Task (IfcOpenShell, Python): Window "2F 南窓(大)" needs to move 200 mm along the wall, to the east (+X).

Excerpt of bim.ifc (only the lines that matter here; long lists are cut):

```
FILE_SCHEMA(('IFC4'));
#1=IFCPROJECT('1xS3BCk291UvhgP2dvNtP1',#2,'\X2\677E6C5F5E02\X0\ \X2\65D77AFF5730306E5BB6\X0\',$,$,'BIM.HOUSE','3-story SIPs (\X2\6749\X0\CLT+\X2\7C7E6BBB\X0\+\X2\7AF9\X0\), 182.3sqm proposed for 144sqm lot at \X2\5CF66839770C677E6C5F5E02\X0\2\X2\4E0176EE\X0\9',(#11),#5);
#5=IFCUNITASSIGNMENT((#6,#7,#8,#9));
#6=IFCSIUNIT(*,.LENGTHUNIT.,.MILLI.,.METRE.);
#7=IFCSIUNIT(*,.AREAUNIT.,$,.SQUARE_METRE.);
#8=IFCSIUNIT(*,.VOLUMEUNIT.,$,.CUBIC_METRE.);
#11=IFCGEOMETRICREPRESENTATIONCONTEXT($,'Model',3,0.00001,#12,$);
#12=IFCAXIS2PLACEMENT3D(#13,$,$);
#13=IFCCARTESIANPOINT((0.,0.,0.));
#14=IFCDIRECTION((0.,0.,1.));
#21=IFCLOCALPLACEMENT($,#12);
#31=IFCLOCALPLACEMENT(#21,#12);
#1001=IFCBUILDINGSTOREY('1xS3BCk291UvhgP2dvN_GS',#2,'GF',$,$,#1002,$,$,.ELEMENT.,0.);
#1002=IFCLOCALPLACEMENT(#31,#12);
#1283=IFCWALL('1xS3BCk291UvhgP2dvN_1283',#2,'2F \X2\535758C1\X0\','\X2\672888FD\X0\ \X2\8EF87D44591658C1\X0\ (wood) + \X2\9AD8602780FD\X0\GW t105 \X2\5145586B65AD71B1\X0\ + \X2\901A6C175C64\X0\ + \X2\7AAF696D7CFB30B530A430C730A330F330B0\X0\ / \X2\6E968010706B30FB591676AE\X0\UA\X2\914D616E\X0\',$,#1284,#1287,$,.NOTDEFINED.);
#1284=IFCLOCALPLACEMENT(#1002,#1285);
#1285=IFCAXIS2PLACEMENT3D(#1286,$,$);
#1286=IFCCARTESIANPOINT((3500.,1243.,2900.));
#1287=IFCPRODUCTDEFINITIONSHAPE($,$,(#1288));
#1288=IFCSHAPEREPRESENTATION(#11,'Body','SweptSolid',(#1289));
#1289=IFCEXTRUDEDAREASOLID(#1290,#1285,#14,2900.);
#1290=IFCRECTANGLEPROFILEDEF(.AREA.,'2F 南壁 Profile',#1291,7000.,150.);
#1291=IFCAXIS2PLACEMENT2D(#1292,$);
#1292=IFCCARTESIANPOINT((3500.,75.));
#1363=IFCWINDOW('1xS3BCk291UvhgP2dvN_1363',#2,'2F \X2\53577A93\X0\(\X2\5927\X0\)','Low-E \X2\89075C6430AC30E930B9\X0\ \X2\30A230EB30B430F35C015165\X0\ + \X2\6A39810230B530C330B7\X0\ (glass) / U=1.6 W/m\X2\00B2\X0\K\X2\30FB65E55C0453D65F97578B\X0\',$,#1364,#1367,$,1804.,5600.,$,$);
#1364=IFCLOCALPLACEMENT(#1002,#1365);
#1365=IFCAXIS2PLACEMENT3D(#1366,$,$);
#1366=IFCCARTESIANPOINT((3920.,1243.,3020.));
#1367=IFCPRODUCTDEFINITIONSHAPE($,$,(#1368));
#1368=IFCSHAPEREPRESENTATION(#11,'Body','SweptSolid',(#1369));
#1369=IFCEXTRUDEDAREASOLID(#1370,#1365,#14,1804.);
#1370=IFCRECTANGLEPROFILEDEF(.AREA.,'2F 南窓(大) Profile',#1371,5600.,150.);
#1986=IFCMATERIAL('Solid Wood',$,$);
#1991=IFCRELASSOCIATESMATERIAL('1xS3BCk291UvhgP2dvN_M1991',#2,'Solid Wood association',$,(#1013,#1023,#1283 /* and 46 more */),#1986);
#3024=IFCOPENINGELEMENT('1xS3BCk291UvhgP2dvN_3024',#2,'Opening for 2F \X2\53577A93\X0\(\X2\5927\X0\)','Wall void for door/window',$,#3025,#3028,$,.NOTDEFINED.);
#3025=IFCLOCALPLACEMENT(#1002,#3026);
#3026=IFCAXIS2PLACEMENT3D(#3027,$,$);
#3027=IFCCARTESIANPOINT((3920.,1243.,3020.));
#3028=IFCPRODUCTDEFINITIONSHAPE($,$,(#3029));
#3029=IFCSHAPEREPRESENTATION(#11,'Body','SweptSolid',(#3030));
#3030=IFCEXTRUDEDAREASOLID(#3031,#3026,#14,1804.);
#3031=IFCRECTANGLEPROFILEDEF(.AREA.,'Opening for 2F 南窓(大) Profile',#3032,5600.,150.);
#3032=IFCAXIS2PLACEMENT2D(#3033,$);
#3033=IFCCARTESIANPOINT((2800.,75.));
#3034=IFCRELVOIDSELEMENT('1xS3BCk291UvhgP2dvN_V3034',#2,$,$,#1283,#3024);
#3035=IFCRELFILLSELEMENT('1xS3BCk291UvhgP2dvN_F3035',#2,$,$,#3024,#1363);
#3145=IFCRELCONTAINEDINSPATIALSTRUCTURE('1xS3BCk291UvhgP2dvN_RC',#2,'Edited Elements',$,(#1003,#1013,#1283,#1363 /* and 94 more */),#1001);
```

```python
import ifcopenshell
import ifcopenshell.api.geometry
import ifcopenshell.util.placement

model = ifcopenshell.open("bim.ifc")

window = model.by_id(1363)
opening = window.FillsVoids[0].RelatingOpeningElement
wall = opening.VoidsElements[0].RelatingBuildingElement

wall_matrix = ifcopenshell.util.placement.get_local_placement(wall.ObjectPlacement)
shift = wall_matrix[:3, 0] * 200.0
before = ifcopenshell.util.placement.get_local_placement(window.ObjectPlacement)[:3, 3].copy()

# The window is not placed relative to its opening, so move both.
for product in (opening, window):
    matrix = ifcopenshell.util.placement.get_local_placement(product.ObjectPlacement)
    matrix[:3, 3] += shift
    ifcopenshell.api.geometry.edit_object_placement(model, product=product, matrix=matrix, is_si=False)

after = ifcopenshell.util.placement.get_local_placement(window.ObjectPlacement)[:3, 3]
print("window moved by", (after - before).round(3) + 0.0)

model.write("bim_edited.ifc")
```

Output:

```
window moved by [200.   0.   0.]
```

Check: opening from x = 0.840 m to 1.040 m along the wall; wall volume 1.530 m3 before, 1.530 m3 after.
